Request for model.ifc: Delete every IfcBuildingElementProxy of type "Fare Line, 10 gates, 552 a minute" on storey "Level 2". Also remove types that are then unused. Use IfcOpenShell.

First a look at what the model holds.

```python
import ifcopenshell
import ifcopenshell.util.element

model = ifcopenshell.open("model.ifc")
print(model.schema)
storey = next(s for s in model.by_type("IfcBuildingStorey") if s.Name == "Level 2")
proxies = [e for e in ifcopenshell.util.element.get_decomposition(storey) if e.is_a("IfcBuildingElementProxy")]
seen = {}
for e in proxies:
    element_type = ifcopenshell.util.element.get_type(e)
    name = element_type.Name if element_type not in (None, e) else None
    seen[name] = seen.get(name, 0) + 1
for name, count in sorted(seen.items(), key=str):
    print(count, "x", name)
```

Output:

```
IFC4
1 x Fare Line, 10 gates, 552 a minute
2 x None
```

```python
import ifcopenshell
import ifcopenshell.api.root
import ifcopenshell.util.element

model = ifcopenshell.open("model.ifc")

storey = next(s for s in model.by_type("IfcBuildingStorey") if s.Name == "Level 2")
proxies = [e for e in ifcopenshell.util.element.get_decomposition(storey) if e.is_a("IfcBuildingElementProxy")]
targets = [e for e in proxies if (t := ifcopenshell.util.element.get_type(e)) not in (None, e) and t.Name == "Fare Line, 10 gates, 552 a minute"]
types = {ifcopenshell.util.element.get_type(e) for e in targets} - {None, *targets}

for e in targets:
    ifcopenshell.api.root.remove_product(model, product=e)
print(len(targets), "removed")

unused = [t for t in types if not ifcopenshell.util.element.get_types(t)]
for t in unused:
    ifcopenshell.api.root.remove_product(model, product=t)
print(len(unused), "unused types removed")

model.write("model-out.ifc")
```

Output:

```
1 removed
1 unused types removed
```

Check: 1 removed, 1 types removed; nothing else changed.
